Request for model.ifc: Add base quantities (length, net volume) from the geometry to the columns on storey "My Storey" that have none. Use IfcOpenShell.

First a look at what the model holds.

```python
import ifcopenshell
import ifcopenshell.util.element
import ifcopenshell.util.unit

model = ifcopenshell.open("model.ifc")
print(model.schema)
for unit_type in ("LENGTHUNIT", "AREAUNIT", "VOLUMEUNIT"):
    print(unit_type, ifcopenshell.util.unit.calculate_unit_scale(model, unit_type))
storey = next(s for s in model.by_type("IfcBuildingStorey") if s.Name == "My Storey")
columns = [e for e in ifcopenshell.util.element.get_decomposition(storey) if e.is_a("IfcColumn")]
for e in sorted(columns, key=lambda e: e.id()):
    print(e.id(), e.is_a(), e.Name, list(ifcopenshell.util.element.get_psets(e, qtos_only=True)), sep=" | ")
```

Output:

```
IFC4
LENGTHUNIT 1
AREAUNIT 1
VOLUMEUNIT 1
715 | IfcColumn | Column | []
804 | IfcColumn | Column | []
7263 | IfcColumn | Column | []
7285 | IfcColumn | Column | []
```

```python
import ifcopenshell
import ifcopenshell.api.pset
import ifcopenshell.geom
import ifcopenshell.util.element
import ifcopenshell.util.shape
import ifcopenshell.util.unit

model = ifcopenshell.open("model.ifc")
unit_scale = ifcopenshell.util.unit.calculate_unit_scale(model)
volume_scale = ifcopenshell.util.unit.calculate_unit_scale(model, "VOLUMEUNIT")
settings = ifcopenshell.geom.settings()

storey = next(s for s in model.by_type("IfcBuildingStorey") if s.Name == "My Storey")
columns = [e for e in ifcopenshell.util.element.get_decomposition(storey) if e.is_a("IfcColumn")]

for e in sorted(columns, key=lambda e: e.id()):
    if ifcopenshell.util.element.get_psets(e, qtos_only=True, should_inherit=False):
        continue
    # Geometry comes back in metres, in the element's own axes.
    shape = ifcopenshell.geom.create_shape(settings, e)
    values = {
        "Length": ifcopenshell.util.shape.get_z(shape.geometry) / unit_scale,
        "NetVolume": ifcopenshell.util.shape.get_volume(shape.geometry) / volume_scale,
    }
    qto = ifcopenshell.api.pset.add_qto(model, product=e, name="Qto_ColumnBaseQuantities")
    ifcopenshell.api.pset.edit_qto(model, qto=qto, properties=values)
    print(e.id(), {k: round(v, 3) for k, v in values.items()})

model.write("model_rev.ifc")
```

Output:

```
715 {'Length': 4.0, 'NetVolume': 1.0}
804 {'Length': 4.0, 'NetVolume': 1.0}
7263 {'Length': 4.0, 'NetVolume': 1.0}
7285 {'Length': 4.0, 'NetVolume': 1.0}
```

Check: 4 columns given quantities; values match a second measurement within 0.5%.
